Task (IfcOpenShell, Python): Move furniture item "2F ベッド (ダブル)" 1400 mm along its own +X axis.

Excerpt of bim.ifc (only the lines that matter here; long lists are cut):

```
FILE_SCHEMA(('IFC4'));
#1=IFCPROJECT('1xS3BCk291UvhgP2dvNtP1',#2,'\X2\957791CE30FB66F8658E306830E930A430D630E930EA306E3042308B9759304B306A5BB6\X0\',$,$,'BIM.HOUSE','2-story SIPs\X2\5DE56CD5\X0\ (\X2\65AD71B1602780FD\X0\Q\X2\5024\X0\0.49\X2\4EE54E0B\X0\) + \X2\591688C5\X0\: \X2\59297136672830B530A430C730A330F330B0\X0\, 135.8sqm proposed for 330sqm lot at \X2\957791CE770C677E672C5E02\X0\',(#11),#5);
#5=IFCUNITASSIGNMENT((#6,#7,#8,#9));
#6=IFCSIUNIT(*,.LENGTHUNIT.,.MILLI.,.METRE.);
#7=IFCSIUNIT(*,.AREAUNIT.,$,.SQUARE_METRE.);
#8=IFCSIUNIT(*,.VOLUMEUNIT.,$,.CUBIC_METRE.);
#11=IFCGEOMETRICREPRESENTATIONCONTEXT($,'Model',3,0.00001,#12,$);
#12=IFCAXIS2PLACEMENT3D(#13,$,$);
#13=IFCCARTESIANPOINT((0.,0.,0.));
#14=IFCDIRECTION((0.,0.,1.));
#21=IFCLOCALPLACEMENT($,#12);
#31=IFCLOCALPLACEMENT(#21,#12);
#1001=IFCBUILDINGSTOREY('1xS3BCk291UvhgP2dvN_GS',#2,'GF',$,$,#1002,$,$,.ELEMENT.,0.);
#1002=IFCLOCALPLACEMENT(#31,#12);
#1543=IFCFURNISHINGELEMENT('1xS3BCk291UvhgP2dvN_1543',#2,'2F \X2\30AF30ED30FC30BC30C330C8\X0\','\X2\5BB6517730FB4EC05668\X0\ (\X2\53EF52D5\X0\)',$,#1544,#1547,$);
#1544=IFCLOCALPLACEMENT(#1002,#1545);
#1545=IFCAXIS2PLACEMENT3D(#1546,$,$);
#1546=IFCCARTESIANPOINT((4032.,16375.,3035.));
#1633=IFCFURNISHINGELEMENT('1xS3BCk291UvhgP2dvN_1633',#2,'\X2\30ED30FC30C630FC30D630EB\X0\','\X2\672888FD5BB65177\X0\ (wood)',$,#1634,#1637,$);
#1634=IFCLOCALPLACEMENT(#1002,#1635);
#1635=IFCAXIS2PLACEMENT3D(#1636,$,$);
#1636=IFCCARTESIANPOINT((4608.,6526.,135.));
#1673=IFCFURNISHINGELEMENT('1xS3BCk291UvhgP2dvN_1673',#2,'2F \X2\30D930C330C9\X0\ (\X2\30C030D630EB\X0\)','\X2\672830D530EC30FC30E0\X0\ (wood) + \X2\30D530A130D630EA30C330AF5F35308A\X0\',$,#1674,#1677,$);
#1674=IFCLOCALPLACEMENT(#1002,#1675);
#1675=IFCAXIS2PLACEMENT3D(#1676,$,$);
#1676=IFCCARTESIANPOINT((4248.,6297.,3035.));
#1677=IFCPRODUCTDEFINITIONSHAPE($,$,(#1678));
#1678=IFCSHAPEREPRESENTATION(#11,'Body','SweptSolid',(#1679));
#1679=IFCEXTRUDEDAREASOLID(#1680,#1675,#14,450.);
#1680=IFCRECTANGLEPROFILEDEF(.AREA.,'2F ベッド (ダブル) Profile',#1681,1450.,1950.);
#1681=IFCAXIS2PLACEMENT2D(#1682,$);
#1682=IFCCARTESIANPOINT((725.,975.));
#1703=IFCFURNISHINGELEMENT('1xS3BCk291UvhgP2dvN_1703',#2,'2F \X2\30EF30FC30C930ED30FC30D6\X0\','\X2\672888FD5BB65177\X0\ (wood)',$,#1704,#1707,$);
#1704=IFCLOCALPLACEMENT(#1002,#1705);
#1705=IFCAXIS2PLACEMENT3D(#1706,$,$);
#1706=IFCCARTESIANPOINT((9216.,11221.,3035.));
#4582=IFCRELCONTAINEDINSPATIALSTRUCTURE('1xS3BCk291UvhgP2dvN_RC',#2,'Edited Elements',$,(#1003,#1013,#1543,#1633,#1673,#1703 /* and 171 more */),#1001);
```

```python
import ifcopenshell
import ifcopenshell.api.geometry
import ifcopenshell.util.placement
import ifcopenshell.util.unit

model = ifcopenshell.open("bim.ifc")
unit_scale = ifcopenshell.util.unit.calculate_unit_scale(model)

item = model.by_id(1673)
matrix = ifcopenshell.util.placement.get_local_placement(item.ObjectPlacement)
matrix[:3, 3] += matrix[:3, 0] * 1.4 / unit_scale
ifcopenshell.api.geometry.edit_object_placement(model, product=item, matrix=matrix, is_si=False)

print(ifcopenshell.util.placement.get_local_placement(item.ObjectPlacement).round(3) + 0.0)

model.write("bim_edited.ifc")
```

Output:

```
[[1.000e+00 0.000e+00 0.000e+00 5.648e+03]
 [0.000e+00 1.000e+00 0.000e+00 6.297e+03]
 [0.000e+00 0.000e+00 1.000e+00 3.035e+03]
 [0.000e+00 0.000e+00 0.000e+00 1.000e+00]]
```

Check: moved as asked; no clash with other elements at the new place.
